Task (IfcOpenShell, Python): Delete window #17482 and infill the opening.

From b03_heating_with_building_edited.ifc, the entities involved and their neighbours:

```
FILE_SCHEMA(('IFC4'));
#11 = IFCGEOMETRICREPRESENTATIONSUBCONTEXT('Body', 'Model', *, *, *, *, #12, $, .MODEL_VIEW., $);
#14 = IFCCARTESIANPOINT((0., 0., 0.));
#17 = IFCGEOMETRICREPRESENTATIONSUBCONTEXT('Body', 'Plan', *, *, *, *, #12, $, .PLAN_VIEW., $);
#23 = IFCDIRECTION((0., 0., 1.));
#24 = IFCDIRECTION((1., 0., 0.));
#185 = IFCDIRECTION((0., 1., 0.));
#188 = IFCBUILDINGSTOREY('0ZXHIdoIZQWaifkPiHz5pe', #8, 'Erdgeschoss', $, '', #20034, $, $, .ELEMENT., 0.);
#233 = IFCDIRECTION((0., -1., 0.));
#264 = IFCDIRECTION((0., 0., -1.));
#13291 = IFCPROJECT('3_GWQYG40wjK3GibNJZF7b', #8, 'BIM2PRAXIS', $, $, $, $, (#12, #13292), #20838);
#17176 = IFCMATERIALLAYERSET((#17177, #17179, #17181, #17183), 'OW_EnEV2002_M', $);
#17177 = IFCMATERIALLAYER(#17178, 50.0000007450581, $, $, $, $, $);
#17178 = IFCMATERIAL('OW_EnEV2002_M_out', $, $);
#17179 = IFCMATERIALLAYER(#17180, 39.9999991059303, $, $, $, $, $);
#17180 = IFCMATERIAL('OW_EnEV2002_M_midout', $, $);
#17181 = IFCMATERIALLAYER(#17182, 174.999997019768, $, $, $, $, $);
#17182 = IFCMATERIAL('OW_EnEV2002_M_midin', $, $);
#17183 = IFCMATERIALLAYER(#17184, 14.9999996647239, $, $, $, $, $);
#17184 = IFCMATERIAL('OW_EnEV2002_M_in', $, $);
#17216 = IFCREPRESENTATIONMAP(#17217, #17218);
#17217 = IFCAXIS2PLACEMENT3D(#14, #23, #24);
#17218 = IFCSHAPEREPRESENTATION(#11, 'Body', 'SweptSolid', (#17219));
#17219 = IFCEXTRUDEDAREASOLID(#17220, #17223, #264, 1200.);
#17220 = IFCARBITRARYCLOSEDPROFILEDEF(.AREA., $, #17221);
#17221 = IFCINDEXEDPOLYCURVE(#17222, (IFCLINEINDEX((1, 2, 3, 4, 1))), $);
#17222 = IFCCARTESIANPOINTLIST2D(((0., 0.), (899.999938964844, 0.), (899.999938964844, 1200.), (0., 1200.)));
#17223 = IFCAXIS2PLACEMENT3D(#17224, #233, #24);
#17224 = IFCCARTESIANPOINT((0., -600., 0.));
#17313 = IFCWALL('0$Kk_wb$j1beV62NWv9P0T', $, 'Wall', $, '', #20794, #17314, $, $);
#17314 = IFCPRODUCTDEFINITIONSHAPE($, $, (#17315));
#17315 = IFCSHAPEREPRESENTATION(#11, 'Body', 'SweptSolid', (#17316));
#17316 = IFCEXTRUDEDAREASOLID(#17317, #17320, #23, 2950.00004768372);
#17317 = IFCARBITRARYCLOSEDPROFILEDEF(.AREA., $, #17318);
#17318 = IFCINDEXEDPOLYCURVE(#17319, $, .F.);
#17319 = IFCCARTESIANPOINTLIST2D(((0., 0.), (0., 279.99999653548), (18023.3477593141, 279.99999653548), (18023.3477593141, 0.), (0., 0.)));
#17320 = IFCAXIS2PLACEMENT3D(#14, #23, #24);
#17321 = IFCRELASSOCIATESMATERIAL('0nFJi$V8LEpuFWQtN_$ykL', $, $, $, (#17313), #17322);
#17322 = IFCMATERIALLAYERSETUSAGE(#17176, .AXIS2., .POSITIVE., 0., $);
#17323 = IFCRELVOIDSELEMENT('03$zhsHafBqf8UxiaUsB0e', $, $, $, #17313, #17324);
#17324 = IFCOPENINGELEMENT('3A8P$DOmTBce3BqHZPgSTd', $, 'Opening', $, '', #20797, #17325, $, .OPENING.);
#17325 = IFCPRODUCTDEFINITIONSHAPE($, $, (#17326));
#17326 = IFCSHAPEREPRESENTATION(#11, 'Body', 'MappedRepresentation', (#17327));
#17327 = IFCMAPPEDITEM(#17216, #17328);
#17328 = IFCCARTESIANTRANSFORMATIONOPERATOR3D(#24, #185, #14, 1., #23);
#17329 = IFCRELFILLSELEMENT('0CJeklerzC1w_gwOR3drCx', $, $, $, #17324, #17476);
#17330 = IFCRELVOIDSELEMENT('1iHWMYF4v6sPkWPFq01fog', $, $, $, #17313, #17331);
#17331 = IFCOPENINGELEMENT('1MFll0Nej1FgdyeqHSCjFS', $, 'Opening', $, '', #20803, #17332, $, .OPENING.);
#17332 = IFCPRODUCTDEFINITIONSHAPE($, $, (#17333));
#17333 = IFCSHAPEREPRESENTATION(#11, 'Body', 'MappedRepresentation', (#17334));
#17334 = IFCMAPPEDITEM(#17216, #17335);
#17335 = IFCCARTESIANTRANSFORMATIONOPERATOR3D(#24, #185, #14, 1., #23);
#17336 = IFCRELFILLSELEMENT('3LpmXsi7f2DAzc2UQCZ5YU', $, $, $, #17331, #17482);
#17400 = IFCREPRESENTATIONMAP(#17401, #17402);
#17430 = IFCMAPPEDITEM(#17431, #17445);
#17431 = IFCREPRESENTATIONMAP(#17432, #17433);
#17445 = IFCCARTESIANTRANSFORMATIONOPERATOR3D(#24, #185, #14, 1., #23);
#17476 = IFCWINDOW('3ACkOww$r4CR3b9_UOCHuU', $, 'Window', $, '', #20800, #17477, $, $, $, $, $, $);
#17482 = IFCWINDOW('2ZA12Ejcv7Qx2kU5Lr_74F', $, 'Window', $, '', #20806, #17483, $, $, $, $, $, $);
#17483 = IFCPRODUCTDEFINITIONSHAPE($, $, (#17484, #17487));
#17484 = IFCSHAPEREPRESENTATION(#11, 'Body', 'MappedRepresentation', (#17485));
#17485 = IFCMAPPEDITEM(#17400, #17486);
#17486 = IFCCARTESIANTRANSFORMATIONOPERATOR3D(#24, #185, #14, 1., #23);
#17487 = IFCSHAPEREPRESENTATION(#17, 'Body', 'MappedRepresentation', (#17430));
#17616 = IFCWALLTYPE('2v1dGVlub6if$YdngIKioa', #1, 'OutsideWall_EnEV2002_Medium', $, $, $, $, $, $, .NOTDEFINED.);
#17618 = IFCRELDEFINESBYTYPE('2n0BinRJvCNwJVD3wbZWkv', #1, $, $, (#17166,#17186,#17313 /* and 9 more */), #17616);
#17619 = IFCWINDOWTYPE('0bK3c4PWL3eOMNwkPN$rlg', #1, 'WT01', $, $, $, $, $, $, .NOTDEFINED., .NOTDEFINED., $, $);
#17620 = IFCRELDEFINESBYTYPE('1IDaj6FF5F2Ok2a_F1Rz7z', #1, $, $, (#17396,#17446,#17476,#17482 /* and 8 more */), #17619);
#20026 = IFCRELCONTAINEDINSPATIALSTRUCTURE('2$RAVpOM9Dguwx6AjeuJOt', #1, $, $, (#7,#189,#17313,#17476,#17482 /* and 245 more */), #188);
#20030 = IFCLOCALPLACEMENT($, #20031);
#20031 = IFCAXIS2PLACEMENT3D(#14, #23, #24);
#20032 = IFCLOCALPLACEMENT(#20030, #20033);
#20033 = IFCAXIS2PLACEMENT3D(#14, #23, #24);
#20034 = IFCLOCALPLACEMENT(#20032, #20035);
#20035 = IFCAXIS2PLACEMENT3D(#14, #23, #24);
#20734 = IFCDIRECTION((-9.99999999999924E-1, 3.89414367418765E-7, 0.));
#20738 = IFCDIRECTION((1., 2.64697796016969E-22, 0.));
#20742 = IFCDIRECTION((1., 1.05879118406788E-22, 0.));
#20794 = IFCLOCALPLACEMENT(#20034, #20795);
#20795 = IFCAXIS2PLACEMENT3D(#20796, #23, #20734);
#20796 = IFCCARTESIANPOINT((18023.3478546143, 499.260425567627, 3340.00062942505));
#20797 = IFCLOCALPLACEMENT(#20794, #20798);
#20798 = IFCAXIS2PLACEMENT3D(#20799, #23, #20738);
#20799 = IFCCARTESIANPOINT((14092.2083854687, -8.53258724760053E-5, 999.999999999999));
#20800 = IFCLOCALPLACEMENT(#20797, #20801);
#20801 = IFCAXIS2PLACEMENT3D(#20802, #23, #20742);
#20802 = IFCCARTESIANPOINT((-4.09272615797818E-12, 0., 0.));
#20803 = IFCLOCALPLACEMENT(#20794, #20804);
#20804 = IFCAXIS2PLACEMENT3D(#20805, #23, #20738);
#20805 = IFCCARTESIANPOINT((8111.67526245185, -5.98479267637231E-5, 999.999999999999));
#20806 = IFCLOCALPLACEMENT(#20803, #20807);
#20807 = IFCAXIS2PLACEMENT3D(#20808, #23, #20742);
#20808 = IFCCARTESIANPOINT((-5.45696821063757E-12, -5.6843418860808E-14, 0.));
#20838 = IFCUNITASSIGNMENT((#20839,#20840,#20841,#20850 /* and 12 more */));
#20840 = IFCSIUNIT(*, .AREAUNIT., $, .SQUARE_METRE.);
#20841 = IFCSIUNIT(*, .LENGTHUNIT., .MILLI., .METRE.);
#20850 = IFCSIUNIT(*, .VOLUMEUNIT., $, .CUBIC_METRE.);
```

```python
import ifcopenshell
import ifcopenshell.api.feature
import ifcopenshell.api.root
import ifcopenshell.geom
import ifcopenshell.util.shape

model = ifcopenshell.open("b03_heating_with_building_edited.ifc")
settings = ifcopenshell.geom.settings()


def volume(element):
    """Net volume in cubic metres, openings subtracted."""
    shape = ifcopenshell.geom.create_shape(settings, element)
    return ifcopenshell.util.shape.get_volume(shape.geometry)


window = model.by_id(17482)
opening = window.FillsVoids[0].RelatingOpeningElement
wall = opening.VoidsElements[0].RelatingBuildingElement
before = volume(wall)

ifcopenshell.api.root.remove_product(model, product=window)
ifcopenshell.api.feature.remove_feature(model, feature=opening)

after = volume(wall)

print(f"wall volume {before:.3f} -> {after:.3f} m3")

model.write("b03_heating_with_building_edited_v2.ifc")
```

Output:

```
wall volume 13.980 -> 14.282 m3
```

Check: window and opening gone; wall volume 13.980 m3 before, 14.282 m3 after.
